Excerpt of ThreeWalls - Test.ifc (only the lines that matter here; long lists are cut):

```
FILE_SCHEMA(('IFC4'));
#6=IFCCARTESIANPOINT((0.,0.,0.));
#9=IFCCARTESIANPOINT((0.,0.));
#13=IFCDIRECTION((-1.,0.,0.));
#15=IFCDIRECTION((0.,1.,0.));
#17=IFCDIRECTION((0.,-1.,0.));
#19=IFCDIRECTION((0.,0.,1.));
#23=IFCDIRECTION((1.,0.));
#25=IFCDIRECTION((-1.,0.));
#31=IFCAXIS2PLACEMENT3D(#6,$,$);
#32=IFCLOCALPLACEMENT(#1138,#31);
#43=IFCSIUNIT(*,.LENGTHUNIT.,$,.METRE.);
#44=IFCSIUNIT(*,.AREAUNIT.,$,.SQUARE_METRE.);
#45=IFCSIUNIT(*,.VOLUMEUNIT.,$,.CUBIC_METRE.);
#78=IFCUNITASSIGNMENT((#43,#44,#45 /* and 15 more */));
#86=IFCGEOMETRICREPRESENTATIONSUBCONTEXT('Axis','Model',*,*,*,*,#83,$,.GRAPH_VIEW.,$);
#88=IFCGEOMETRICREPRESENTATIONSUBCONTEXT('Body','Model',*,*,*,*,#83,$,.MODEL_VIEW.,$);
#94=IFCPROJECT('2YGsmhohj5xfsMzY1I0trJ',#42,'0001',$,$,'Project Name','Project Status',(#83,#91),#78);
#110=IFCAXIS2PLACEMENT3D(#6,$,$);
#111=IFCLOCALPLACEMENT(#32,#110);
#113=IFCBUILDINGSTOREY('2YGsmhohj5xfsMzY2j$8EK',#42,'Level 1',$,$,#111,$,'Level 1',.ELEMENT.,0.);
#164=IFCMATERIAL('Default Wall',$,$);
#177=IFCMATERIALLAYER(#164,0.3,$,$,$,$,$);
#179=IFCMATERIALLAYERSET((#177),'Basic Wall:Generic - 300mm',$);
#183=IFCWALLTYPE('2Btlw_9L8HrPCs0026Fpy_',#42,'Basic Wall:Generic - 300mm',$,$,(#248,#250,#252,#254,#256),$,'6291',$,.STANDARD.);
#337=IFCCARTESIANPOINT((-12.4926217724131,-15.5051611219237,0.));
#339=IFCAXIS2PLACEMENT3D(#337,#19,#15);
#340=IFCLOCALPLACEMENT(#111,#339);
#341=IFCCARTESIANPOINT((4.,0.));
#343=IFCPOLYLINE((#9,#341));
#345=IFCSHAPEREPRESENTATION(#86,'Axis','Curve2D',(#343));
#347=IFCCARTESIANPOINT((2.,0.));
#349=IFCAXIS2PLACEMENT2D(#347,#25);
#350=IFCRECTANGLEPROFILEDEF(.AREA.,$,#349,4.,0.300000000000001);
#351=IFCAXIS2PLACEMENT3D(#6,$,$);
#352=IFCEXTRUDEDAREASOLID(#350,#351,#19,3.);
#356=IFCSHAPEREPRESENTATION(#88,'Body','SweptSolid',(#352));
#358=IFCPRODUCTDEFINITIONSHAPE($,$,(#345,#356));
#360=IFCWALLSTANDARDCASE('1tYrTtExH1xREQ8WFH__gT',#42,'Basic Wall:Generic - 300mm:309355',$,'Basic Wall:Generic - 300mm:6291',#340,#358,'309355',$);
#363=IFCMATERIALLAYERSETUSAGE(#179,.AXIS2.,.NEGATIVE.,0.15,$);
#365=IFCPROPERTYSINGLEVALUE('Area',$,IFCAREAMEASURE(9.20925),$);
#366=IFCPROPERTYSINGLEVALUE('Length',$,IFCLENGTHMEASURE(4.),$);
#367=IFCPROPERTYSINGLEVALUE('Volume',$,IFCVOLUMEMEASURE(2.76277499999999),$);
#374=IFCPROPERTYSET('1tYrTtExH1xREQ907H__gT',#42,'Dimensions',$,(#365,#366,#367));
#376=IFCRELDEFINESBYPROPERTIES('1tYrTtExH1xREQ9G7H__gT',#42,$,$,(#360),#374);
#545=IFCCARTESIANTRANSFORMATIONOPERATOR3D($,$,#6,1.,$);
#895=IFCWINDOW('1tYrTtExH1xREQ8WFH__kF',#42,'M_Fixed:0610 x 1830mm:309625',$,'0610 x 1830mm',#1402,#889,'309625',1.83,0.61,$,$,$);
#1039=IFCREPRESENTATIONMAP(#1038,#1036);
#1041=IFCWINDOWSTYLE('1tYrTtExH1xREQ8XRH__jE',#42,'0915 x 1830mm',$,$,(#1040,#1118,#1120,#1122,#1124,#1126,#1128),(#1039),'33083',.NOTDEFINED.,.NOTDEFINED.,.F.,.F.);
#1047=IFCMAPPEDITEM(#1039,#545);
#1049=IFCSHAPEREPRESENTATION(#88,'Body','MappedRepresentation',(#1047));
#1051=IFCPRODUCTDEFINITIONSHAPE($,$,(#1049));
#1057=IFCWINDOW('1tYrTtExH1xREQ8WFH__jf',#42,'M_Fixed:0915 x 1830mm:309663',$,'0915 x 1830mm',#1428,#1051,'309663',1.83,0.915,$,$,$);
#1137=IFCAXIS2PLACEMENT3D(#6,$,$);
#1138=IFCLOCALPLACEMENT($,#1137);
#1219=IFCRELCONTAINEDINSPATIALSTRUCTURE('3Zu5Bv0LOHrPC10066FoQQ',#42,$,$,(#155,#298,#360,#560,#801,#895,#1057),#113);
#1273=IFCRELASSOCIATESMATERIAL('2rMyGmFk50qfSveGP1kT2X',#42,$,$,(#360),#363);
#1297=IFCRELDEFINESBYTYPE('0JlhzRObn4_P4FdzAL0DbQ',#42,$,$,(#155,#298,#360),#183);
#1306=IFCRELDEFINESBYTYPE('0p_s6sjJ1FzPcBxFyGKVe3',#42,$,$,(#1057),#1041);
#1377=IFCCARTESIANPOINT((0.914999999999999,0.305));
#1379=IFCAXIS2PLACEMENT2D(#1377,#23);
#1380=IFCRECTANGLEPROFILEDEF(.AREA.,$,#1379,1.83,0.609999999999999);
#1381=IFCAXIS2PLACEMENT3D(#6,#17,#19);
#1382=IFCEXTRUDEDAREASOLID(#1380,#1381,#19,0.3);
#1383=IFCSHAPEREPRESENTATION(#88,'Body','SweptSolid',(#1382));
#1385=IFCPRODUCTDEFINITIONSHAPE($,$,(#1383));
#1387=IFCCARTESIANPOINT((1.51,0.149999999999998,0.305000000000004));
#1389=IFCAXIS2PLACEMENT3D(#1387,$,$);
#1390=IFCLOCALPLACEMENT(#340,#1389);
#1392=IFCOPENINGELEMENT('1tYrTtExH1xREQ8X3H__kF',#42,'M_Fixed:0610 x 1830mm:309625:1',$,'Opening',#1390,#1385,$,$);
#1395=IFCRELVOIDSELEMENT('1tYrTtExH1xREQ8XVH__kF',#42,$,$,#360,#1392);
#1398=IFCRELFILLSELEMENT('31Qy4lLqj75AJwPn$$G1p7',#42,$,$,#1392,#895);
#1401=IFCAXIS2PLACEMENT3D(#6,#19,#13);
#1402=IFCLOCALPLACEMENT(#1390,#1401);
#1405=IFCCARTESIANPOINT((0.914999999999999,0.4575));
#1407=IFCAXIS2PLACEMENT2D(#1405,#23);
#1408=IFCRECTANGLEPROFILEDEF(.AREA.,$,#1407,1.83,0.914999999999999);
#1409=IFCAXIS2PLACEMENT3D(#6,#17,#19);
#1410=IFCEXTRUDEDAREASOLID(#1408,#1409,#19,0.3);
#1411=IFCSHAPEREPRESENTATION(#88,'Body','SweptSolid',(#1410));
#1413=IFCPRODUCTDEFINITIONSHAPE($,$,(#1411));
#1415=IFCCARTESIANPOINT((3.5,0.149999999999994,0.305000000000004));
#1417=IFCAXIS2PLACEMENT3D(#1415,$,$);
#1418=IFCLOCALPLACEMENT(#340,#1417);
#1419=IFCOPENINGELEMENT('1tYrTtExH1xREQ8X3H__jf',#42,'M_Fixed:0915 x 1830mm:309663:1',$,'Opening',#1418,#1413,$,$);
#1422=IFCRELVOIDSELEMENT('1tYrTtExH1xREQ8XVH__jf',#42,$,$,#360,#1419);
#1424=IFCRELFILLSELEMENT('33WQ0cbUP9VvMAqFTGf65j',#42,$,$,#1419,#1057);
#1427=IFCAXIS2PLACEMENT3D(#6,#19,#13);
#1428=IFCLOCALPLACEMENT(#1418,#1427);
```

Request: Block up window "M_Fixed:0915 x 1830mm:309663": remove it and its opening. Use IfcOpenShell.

```python
import ifcopenshell
import ifcopenshell.api.feature
import ifcopenshell.api.pset
import ifcopenshell.api.root
import ifcopenshell.geom
import ifcopenshell.util.element
import ifcopenshell.util.shape
import ifcopenshell.util.unit

model = ifcopenshell.open("ThreeWalls - Test.ifc")
area_scale = ifcopenshell.util.unit.calculate_unit_scale(model, "AREAUNIT")
volume_scale = ifcopenshell.util.unit.calculate_unit_scale(model, "VOLUMEUNIT")
settings = ifcopenshell.geom.settings()


def volume(element):
    """Net volume in cubic metres, openings subtracted."""
    shape = ifcopenshell.geom.create_shape(settings, element)
    return ifcopenshell.util.shape.get_volume(shape.geometry)


window = model.by_guid("1tYrTtExH1xREQ8WFH__jf")
opening = window.FillsVoids[0].RelatingOpeningElement
wall = opening.VoidsElements[0].RelatingBuildingElement
before = volume(wall)

ifcopenshell.api.root.remove_product(model, product=window)
ifcopenshell.api.feature.remove_feature(model, feature=opening)

after = volume(wall)
thickness = 0.3  # wall thickness in metres

# Update the wall's stored quantities.
pset = model.by_id(ifcopenshell.util.element.get_pset(wall, "Dimensions", should_inherit=False)["id"])
ifcopenshell.api.pset.edit_pset(model, pset=pset, properties={
    "Area": model.create_entity("IfcAreaMeasure", after / thickness / area_scale),
    "Volume": model.create_entity("IfcVolumeMeasure", after / volume_scale),
})

print(f"wall volume {before:.3f} -> {after:.3f} m3")

model.write("ThreeWalls - Test-out.ifc")
```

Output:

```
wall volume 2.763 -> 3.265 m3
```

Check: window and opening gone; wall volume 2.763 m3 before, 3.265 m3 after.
